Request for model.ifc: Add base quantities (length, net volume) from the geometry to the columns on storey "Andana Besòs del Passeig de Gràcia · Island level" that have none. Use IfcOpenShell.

First a look at what the model holds.

```python
import ifcopenshell
import ifcopenshell.util.element
import ifcopenshell.util.unit

model = ifcopenshell.open("model.ifc")
print(model.schema)
for unit_type in ("LENGTHUNIT", "AREAUNIT", "VOLUMEUNIT"):
    print(unit_type, ifcopenshell.util.unit.calculate_unit_scale(model, unit_type))
storey = next(s for s in model.by_type("IfcBuildingStorey") if s.Name == "Andana Besòs del Passeig de Gràcia · Island level")
columns = [e for e in ifcopenshell.util.element.get_decomposition(storey) if e.is_a("IfcColumn")]
for e in sorted(columns, key=lambda e: e.id()):
    print(e.id(), e.is_a(), e.Name, list(ifcopenshell.util.element.get_psets(e, qtos_only=True)), sep=" | ")
```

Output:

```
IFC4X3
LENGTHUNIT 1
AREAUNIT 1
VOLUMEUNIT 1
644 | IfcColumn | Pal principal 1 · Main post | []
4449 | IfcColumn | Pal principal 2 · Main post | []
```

```python
import ifcopenshell
import ifcopenshell.api.pset
import ifcopenshell.geom
import ifcopenshell.util.element
import ifcopenshell.util.shape
import ifcopenshell.util.unit

model = ifcopenshell.open("model.ifc")
unit_scale = ifcopenshell.util.unit.calculate_unit_scale(model)
volume_scale = ifcopenshell.util.unit.calculate_unit_scale(model, "VOLUMEUNIT")
settings = ifcopenshell.geom.settings()

storey = next(s for s in model.by_type("IfcBuildingStorey") if s.Name == "Andana Besòs del Passeig de Gràcia · Island level")
columns = [e for e in ifcopenshell.util.element.get_decomposition(storey) if e.is_a("IfcColumn")]

for e in sorted(columns, key=lambda e: e.id()):
    if ifcopenshell.util.element.get_psets(e, qtos_only=True, should_inherit=False):
        continue
    # Geometry comes back in metres, in the element's own axes.
    shape = ifcopenshell.geom.create_shape(settings, e)
    values = {
        "Length": ifcopenshell.util.shape.get_z(shape.geometry) / unit_scale,
        "NetVolume": ifcopenshell.util.shape.get_volume(shape.geometry) / volume_scale,
    }
    qto = ifcopenshell.api.pset.add_qto(model, product=e, name="Qto_ColumnBaseQuantities")
    ifcopenshell.api.pset.edit_qto(model, qto=qto, properties=values)
    print(e.id(), {k: round(v, 3) for k, v in values.items()})

model.write("model_rev.ifc")
```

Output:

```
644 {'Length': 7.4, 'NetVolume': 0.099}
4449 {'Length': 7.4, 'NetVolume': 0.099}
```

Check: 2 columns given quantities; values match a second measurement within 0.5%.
